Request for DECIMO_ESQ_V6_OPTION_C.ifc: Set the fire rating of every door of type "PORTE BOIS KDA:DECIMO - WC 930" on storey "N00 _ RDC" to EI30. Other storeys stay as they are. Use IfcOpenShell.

First a look at what the model holds.

```python
import ifcopenshell
import ifcopenshell.util.element

model = ifcopenshell.open("DECIMO_ESQ_V6_OPTION_C.ifc")
print(model.schema)
storey = next(s for s in model.by_type("IfcBuildingStorey") if s.Name == "N00 _ RDC")
doors = [e for e in ifcopenshell.util.element.get_decomposition(storey) if e.is_a("IfcDoor")]
seen = {}
for e in doors:
    element_type = ifcopenshell.util.element.get_type(e)
    key = (element_type.Name if element_type != e and element_type else None, ifcopenshell.util.element.get_pset(e, "Pset_DoorCommon", "FireRating"))
    seen[key] = seen.get(key, 0) + 1
for (name, value), count in sorted(seen.items(), key=str):
    print(count, "x", name, "|", value)
```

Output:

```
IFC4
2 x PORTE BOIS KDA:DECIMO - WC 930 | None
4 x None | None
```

```python
import ifcopenshell
import ifcopenshell.api.pset
import ifcopenshell.util.element

model = ifcopenshell.open("DECIMO_ESQ_V6_OPTION_C.ifc")

storey = next(s for s in model.by_type("IfcBuildingStorey") if s.Name == "N00 _ RDC")
doors = [e for e in ifcopenshell.util.element.get_decomposition(storey) if e.is_a("IfcDoor")]

count = 0
for e in doors:
    element_type = ifcopenshell.util.element.get_type(e)
    if element_type in (None, e) or element_type.Name != "PORTE BOIS KDA:DECIMO - WC 930":
        continue
    # add_pset returns the element's existing set when there is one.
    pset = ifcopenshell.api.pset.add_pset(model, product=e, name="Pset_DoorCommon")
    ifcopenshell.api.pset.edit_pset(model, pset=pset, properties={"FireRating": "EI30"})
    count += 1

print(count, "doors updated")

model.write("DECIMO_ESQ_V6_OPTION_C-out.ifc")
```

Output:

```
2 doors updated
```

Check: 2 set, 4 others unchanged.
